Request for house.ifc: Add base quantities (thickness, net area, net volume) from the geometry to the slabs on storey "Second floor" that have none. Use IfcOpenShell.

First a look at what the model holds.

```python
import ifcopenshell
import ifcopenshell.util.element
import ifcopenshell.util.unit

model = ifcopenshell.open("house.ifc")
print(model.schema)
for unit_type in ("LENGTHUNIT", "AREAUNIT", "VOLUMEUNIT"):
    print(unit_type, ifcopenshell.util.unit.calculate_unit_scale(model, unit_type))
storey = next(s for s in model.by_type("IfcBuildingStorey") if s.Name == "Second floor")
slabs = [e for e in ifcopenshell.util.element.get_decomposition(storey) if e.is_a("IfcSlab")]
for e in sorted(slabs, key=lambda e: e.id()):
    print(e.id(), e.is_a(), e.Name, list(ifcopenshell.util.element.get_psets(e, qtos_only=True)), sep=" | ")
```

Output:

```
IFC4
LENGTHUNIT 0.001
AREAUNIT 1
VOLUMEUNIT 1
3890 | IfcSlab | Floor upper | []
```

```python
import ifcopenshell
import ifcopenshell.api.pset
import ifcopenshell.geom
import ifcopenshell.util.element
import ifcopenshell.util.shape
import ifcopenshell.util.unit

model = ifcopenshell.open("house.ifc")
unit_scale = ifcopenshell.util.unit.calculate_unit_scale(model)
area_scale = ifcopenshell.util.unit.calculate_unit_scale(model, "AREAUNIT")
volume_scale = ifcopenshell.util.unit.calculate_unit_scale(model, "VOLUMEUNIT")
settings = ifcopenshell.geom.settings()

storey = next(s for s in model.by_type("IfcBuildingStorey") if s.Name == "Second floor")
slabs = [e for e in ifcopenshell.util.element.get_decomposition(storey) if e.is_a("IfcSlab")]

for e in sorted(slabs, key=lambda e: e.id()):
    if ifcopenshell.util.element.get_psets(e, qtos_only=True, should_inherit=False):
        continue
    # Geometry comes back in metres, in the element's own axes.
    shape = ifcopenshell.geom.create_shape(settings, e)
    values = {
        "Width": ifcopenshell.util.shape.get_z(shape.geometry) / unit_scale,
        "NetArea": ifcopenshell.util.shape.get_footprint_area(shape.geometry) / area_scale,
        "NetVolume": ifcopenshell.util.shape.get_volume(shape.geometry) / volume_scale,
    }
    qto = ifcopenshell.api.pset.add_qto(model, product=e, name="Qto_SlabBaseQuantities")
    ifcopenshell.api.pset.edit_qto(model, qto=qto, properties=values)
    print(e.id(), {k: round(v, 3) for k, v in values.items()})

model.write("house_v2.ifc")
```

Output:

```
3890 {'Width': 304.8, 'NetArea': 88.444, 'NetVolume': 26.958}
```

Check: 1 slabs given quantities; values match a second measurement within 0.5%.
